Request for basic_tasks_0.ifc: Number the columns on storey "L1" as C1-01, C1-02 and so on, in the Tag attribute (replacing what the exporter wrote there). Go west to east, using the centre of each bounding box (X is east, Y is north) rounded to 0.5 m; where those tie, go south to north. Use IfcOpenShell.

First a look at what the model holds.

```python
import ifcopenshell
import ifcopenshell.util.element
import ifcopenshell.util.placement

model = ifcopenshell.open("basic_tasks_0.ifc")
print(model.schema)
storey = next(s for s in model.by_type("IfcBuildingStorey") if s.Name == "L1")
columns = [e for e in ifcopenshell.util.element.get_decomposition(storey) if e.is_a("IfcColumn")]
for e in sorted(columns, key=lambda e: e.id()):
    origin = ifcopenshell.util.placement.get_local_placement(e.ObjectPlacement)[:3, 3]
    print(e.id(), e.Tag, e.Name, origin.round(2) + 0.0, sep=" | ")
```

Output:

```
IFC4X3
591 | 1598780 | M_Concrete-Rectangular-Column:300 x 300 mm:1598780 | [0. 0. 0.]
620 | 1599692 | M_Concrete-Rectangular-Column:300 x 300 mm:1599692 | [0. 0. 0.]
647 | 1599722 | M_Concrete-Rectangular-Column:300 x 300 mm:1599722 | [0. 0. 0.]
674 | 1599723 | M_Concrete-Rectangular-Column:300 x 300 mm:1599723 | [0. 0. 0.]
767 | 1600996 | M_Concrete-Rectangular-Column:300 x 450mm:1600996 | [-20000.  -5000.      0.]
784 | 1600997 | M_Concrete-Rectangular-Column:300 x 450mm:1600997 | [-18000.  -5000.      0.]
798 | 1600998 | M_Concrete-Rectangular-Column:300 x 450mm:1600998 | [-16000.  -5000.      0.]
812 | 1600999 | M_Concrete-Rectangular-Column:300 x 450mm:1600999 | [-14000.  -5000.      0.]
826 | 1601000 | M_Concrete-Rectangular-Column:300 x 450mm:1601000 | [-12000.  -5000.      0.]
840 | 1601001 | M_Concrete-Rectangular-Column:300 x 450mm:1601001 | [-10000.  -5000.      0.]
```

```python
import ifcopenshell
import ifcopenshell.geom
import ifcopenshell.util.element
import ifcopenshell.util.shape

model = ifcopenshell.open("basic_tasks_0.ifc")
settings = ifcopenshell.geom.settings()
settings.set("use-world-coords", True)


def centre(element):
    shape = ifcopenshell.geom.create_shape(settings, element)
    return ifcopenshell.util.shape.get_bbox_centroid(shape.geometry)


storey = next(s for s in model.by_type("IfcBuildingStorey") if s.Name == "L1")
columns = [e for e in ifcopenshell.util.element.get_decomposition(storey) if e.is_a("IfcColumn")]

# Insertion points can sit at a corner or the storey origin, so sort by the geometry (in metres).
centres = {e: centre(e) for e in columns}
columns.sort(key=lambda e: (round(centres[e][0] / 0.5), centres[e][1]))

for i, e in enumerate(columns, start=1):
    number = f"C1-{i:02d}"
    e.Tag = number
    print(e.id(), number)

model.write("basic_tasks_0-out.ifc")
```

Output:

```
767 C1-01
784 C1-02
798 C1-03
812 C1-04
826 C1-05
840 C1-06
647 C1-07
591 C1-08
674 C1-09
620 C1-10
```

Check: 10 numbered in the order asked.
